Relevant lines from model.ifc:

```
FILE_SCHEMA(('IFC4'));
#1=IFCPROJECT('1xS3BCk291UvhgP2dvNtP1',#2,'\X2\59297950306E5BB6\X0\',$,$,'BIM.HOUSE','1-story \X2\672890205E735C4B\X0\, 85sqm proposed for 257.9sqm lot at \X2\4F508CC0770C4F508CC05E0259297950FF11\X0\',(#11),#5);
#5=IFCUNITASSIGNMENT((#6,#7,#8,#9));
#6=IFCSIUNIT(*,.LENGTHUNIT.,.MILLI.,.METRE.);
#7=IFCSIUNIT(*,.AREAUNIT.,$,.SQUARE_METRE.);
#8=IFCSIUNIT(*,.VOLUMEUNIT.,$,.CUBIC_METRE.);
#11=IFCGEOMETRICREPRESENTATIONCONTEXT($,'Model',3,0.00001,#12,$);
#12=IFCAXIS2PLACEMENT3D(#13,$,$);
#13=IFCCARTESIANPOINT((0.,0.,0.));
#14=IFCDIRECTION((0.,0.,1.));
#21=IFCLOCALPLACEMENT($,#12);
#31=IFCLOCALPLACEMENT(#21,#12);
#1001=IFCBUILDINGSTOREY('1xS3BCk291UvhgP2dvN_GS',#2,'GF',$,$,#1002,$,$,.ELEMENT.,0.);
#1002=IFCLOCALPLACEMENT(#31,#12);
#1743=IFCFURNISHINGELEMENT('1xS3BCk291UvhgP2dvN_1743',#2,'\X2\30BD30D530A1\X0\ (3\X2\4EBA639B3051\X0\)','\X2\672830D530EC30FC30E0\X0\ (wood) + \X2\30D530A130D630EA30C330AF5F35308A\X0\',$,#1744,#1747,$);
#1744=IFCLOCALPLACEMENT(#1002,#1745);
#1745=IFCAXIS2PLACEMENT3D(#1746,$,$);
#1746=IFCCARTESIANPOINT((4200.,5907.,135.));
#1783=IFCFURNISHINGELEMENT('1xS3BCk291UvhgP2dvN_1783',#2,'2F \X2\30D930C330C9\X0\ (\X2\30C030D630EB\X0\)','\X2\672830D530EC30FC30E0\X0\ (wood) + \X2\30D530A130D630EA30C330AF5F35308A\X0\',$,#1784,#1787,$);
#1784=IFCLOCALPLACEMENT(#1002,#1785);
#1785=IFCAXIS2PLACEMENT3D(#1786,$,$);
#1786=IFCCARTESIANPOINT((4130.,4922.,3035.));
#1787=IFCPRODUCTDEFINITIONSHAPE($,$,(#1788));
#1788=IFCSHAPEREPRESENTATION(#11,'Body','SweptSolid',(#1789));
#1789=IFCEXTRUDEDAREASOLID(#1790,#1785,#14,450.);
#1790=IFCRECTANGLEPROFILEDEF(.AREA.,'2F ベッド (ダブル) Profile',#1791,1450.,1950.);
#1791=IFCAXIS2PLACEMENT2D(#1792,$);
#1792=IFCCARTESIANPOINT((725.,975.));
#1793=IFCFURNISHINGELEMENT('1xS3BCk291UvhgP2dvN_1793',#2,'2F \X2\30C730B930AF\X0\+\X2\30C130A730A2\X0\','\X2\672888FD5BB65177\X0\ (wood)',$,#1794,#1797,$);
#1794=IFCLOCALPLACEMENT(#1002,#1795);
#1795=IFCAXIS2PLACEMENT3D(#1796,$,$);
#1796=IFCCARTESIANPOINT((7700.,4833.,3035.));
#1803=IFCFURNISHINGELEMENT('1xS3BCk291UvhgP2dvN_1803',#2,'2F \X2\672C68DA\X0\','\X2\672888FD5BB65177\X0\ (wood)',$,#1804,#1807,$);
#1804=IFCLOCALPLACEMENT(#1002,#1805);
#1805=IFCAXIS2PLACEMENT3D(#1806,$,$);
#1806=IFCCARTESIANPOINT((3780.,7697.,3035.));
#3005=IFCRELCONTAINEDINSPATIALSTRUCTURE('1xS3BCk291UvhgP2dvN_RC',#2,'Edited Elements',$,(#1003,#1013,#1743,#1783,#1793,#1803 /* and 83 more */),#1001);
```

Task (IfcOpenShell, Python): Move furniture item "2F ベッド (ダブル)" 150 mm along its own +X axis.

```python
import ifcopenshell
import ifcopenshell.api.geometry
import ifcopenshell.util.placement
import ifcopenshell.util.unit

model = ifcopenshell.open("model.ifc")
unit_scale = ifcopenshell.util.unit.calculate_unit_scale(model)

item = model.by_guid("1xS3BCk291UvhgP2dvN_1783")
matrix = ifcopenshell.util.placement.get_local_placement(item.ObjectPlacement)
matrix[:3, 3] += matrix[:3, 0] * 0.15 / unit_scale
ifcopenshell.api.geometry.edit_object_placement(model, product=item, matrix=matrix, is_si=False)

print(ifcopenshell.util.placement.get_local_placement(item.ObjectPlacement).round(3) + 0.0)

model.write("model-out.ifc")
```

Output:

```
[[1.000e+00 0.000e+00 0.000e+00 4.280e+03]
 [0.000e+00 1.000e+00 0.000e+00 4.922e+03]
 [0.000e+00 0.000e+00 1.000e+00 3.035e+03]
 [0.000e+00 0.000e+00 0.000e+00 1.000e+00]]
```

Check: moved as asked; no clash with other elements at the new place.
